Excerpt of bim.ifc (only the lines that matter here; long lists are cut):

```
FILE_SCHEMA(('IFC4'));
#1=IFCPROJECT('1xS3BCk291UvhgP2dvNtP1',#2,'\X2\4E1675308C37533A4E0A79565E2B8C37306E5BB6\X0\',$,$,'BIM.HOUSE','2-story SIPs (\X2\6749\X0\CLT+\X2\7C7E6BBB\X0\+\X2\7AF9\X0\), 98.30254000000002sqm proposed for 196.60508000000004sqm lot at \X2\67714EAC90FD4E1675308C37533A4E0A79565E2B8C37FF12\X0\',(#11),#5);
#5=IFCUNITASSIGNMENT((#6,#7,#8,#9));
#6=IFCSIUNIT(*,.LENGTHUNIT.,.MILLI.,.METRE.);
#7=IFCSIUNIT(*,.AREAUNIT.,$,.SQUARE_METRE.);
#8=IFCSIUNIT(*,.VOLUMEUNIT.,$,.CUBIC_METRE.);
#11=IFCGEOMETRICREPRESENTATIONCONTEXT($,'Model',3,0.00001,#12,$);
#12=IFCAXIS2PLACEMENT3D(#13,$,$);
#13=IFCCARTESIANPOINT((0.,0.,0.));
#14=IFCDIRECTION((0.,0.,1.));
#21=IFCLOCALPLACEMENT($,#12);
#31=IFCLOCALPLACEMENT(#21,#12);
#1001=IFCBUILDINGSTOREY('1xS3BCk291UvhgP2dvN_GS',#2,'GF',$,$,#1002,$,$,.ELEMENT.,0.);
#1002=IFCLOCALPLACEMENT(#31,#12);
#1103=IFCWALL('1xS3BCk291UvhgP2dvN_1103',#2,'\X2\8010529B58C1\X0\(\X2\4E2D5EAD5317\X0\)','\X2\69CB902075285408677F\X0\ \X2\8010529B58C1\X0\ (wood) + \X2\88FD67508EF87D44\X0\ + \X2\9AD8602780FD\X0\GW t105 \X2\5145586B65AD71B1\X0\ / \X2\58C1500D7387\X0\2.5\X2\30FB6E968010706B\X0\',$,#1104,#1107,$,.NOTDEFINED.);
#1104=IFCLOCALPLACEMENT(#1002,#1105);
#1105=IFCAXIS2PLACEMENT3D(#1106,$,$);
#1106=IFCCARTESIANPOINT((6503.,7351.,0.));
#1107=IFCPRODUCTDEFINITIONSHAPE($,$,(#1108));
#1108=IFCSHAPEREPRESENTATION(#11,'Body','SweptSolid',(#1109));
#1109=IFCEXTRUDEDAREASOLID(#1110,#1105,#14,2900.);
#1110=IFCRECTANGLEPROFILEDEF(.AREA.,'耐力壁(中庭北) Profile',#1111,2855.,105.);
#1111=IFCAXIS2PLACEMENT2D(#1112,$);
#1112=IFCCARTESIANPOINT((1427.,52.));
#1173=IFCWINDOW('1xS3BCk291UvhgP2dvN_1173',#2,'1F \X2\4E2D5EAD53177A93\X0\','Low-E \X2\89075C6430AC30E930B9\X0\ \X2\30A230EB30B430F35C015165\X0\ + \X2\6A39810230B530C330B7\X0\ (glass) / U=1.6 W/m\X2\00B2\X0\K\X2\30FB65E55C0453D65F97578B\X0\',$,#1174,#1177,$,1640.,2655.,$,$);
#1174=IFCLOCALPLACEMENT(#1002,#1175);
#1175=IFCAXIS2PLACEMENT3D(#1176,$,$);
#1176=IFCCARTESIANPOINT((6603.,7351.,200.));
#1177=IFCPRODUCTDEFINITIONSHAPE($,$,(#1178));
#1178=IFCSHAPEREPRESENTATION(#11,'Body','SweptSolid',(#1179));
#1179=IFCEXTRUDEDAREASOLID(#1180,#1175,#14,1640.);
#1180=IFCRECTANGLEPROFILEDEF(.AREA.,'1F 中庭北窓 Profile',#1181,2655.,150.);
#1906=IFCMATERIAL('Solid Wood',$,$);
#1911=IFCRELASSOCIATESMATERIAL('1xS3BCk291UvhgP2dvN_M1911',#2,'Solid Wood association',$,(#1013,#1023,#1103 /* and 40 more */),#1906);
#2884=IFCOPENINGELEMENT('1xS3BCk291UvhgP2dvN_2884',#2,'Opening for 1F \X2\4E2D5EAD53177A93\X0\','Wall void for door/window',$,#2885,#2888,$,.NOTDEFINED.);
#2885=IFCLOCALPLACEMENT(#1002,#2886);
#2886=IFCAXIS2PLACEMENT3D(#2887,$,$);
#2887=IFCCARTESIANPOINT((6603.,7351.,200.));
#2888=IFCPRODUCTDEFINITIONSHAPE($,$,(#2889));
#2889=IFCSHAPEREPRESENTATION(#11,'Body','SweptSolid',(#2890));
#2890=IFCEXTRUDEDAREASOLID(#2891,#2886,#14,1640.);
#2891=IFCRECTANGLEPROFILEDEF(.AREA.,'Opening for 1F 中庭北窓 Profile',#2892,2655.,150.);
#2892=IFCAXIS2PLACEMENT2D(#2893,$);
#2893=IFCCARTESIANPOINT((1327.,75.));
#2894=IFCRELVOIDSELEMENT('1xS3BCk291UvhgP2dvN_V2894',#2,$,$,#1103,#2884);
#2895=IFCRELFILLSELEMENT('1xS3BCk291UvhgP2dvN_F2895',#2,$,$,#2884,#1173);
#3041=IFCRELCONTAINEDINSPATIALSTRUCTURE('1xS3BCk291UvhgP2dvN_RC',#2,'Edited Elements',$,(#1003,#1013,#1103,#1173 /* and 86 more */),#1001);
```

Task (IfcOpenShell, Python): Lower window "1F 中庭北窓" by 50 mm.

```python
import numpy as np
import ifcopenshell
import ifcopenshell.api.geometry
import ifcopenshell.util.placement
import ifcopenshell.util.unit

model = ifcopenshell.open("bim.ifc")
unit_scale = ifcopenshell.util.unit.calculate_unit_scale(model)

window = model.by_id(1173)
opening = window.FillsVoids[0].RelatingOpeningElement
dz = -0.05 / unit_scale

shift = np.array([0.0, 0.0, dz])
# The window is not placed relative to its opening, so move both.
for product in (opening, window):
    matrix = ifcopenshell.util.placement.get_local_placement(product.ObjectPlacement)
    matrix[:3, 3] += shift
    ifcopenshell.api.geometry.edit_object_placement(model, product=product, matrix=matrix, is_si=False)

print(f"moved by {dz * unit_scale:+.3f} m")

model.write("bim_updated.ifc")
```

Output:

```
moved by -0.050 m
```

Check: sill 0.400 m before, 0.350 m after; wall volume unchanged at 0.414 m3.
